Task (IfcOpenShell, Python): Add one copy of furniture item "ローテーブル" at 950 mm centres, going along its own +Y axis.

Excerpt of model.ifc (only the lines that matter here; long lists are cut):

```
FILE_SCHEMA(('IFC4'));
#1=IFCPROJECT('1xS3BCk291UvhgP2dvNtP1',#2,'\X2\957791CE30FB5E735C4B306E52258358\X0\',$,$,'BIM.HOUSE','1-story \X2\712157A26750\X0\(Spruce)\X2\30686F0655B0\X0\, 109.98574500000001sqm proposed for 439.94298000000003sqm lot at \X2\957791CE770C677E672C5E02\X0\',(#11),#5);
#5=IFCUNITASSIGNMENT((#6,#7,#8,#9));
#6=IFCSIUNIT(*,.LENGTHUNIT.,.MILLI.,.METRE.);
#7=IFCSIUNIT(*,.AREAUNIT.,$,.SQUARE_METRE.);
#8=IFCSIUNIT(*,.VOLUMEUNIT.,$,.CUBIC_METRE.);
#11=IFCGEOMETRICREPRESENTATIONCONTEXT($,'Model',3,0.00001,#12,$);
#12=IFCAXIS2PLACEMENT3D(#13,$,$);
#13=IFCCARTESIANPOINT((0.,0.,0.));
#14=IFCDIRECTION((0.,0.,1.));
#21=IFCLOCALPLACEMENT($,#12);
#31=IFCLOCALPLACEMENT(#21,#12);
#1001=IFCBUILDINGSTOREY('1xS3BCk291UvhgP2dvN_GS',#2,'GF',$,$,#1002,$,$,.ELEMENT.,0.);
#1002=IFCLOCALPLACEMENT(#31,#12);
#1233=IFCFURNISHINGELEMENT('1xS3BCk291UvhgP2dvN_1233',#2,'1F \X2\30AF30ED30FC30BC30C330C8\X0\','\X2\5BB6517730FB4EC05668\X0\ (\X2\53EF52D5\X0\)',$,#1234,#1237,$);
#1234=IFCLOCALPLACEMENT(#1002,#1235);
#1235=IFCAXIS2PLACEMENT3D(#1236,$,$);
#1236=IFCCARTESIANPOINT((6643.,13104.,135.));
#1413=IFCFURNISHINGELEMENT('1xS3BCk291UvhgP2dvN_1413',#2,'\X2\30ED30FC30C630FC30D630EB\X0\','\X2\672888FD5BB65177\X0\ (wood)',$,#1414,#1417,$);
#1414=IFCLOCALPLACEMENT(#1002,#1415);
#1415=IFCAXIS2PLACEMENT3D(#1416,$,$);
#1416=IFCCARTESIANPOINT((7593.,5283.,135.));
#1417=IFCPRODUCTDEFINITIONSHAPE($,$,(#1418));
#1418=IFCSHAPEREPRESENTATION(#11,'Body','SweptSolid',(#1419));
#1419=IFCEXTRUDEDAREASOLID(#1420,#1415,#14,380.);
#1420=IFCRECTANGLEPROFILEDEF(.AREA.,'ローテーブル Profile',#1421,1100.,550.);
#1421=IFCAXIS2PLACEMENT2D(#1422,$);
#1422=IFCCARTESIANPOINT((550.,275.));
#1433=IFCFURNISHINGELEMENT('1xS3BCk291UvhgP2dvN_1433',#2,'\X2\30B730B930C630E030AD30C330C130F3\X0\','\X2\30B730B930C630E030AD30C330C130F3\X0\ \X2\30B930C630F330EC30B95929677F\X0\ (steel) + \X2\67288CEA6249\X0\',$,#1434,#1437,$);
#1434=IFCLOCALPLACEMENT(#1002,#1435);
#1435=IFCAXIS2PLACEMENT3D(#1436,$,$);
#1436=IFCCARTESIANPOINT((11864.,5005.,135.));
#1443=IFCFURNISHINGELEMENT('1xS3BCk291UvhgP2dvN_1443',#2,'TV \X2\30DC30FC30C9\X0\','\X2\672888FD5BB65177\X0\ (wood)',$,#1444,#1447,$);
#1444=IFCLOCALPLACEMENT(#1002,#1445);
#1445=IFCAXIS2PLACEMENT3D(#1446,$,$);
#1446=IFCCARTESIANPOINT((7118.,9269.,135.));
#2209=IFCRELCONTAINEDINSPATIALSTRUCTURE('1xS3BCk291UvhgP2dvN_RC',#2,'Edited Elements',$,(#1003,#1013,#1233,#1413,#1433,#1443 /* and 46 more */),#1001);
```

```python
import ifcopenshell
import ifcopenshell.api.geometry
import ifcopenshell.api.root
import ifcopenshell.util.element
import ifcopenshell.util.placement
import ifcopenshell.util.unit

model = ifcopenshell.open("model.ifc")
unit_scale = ifcopenshell.util.unit.calculate_unit_scale(model)


def reuse_history(source, copy):
    """copy_class also copies each property set's owner history, people and application; keep the originals."""
    for rel in copy.IsDefinedBy:
        if rel.is_a("IfcRelDefinesByProperties") and (history := rel.RelatingPropertyDefinition.OwnerHistory):
            rel.RelatingPropertyDefinition.OwnerHistory = source.OwnerHistory
            ifcopenshell.util.element.remove_deep2(model, history)


source = model.by_guid("1xS3BCk291UvhgP2dvN_1413")
base = ifcopenshell.util.placement.get_local_placement(source.ObjectPlacement)
step = base[:3, 1] * 0.95 / unit_scale

for i in range(1, 2):
    copy = ifcopenshell.api.root.copy_class(model, product=source)
    copy.Representation = ifcopenshell.util.element.copy_deep(
        model, source.Representation, exclude=["IfcGeometricRepresentationContext", "IfcRepresentationMap"]
    )
    reuse_history(source, copy)
    matrix = base.copy()
    matrix[:3, 3] += i * step
    print("added at", matrix[:3, 3].round(3) + 0.0)
    ifcopenshell.api.geometry.edit_object_placement(model, product=copy, matrix=matrix, is_si=False)

model.write("model-out.ifc")
```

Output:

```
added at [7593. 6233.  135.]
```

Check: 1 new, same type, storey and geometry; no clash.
